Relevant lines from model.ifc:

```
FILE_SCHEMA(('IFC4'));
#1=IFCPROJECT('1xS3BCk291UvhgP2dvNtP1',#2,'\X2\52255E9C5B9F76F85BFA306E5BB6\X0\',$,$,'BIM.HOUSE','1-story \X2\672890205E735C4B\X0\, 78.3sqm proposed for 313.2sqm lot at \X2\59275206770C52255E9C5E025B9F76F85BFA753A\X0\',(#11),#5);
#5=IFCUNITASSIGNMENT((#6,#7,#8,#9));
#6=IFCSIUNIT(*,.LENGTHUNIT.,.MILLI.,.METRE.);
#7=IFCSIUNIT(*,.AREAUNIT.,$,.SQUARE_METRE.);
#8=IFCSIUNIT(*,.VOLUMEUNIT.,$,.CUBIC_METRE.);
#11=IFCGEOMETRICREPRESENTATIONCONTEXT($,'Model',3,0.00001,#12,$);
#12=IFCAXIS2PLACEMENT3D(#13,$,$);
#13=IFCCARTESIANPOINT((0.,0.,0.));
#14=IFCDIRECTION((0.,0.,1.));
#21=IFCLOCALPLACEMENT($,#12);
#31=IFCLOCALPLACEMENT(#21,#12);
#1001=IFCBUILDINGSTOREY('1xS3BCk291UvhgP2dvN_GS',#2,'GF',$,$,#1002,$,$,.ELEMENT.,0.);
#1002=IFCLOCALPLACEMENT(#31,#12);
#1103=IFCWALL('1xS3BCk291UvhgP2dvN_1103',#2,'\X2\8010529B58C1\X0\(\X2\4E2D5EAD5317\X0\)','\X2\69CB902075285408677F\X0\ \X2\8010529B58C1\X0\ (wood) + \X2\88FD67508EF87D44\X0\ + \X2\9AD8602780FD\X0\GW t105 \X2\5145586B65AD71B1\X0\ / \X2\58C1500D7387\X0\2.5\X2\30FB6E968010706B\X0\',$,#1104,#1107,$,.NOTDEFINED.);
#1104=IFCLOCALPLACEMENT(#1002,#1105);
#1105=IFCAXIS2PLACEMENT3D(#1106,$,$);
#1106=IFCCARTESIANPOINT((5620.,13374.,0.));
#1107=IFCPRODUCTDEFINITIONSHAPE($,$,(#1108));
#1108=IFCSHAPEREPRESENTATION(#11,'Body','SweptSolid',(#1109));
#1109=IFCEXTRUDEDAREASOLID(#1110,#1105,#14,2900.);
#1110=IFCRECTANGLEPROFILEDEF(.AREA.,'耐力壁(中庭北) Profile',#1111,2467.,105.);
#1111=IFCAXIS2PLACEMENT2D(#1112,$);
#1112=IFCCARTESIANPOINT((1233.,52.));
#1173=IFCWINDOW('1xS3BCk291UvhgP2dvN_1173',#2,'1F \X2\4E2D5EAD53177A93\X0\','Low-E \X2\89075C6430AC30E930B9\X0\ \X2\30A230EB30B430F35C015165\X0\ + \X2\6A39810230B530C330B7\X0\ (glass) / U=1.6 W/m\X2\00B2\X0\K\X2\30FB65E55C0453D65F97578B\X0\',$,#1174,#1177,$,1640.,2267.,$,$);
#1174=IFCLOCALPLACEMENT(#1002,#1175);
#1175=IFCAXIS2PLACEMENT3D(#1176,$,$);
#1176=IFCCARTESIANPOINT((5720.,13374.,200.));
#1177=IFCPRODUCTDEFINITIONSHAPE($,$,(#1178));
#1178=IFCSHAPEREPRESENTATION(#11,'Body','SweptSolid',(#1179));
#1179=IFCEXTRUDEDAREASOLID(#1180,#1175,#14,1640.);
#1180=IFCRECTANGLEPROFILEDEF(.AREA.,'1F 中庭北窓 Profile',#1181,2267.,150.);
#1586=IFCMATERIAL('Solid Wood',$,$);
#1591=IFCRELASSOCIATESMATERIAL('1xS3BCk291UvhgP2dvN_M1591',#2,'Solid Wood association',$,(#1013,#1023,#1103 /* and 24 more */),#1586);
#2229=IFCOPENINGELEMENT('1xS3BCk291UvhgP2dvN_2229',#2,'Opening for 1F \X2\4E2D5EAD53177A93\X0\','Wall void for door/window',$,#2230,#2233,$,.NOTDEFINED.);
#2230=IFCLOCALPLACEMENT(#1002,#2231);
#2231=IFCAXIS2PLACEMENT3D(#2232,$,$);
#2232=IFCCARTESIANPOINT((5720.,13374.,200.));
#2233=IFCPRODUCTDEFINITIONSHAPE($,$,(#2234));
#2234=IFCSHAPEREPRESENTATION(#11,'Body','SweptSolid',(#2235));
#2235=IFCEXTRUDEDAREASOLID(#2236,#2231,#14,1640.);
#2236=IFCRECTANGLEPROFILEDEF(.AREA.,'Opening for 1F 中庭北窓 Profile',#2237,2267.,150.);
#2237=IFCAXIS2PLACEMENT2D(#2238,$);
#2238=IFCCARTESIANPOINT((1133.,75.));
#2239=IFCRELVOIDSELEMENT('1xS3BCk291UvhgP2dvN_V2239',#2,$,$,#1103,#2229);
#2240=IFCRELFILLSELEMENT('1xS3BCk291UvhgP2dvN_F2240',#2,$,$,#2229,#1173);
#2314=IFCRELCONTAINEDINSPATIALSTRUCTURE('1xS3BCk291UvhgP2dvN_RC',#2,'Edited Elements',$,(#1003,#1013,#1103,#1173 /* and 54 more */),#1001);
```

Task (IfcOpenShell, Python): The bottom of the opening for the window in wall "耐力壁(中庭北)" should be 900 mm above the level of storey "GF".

```python
import numpy as np
import ifcopenshell
import ifcopenshell.api.geometry
import ifcopenshell.geom
import ifcopenshell.util.element
import ifcopenshell.util.placement
import ifcopenshell.util.shape
import ifcopenshell.util.unit

model = ifcopenshell.open("model.ifc")
unit_scale = ifcopenshell.util.unit.calculate_unit_scale(model)

window = model.by_id(1173)
opening = window.FillsVoids[0].RelatingOpeningElement
storey = ifcopenshell.util.element.get_container(window, ifc_class="IfcBuildingStorey")
level = ifcopenshell.util.placement.get_local_placement(storey.ObjectPlacement)[2, 3]

# The opening's origin need not be at the sill, so measure its lowest point.
shape = ifcopenshell.geom.create_shape(ifcopenshell.geom.settings(), opening)
bottom = ifcopenshell.util.shape.get_shape_bottom_elevation(shape, shape.geometry) / unit_scale
dz = level + 0.9 / unit_scale - bottom

shift = np.array([0.0, 0.0, dz])
# The window is not placed relative to its opening, so move both.
for product in (opening, window):
    matrix = ifcopenshell.util.placement.get_local_placement(product.ObjectPlacement)
    matrix[:3, 3] += shift
    ifcopenshell.api.geometry.edit_object_placement(model, product=product, matrix=matrix, is_si=False)

print(f"moved by {dz * unit_scale:+.3f} m")

model.write("model_updated.ifc")
```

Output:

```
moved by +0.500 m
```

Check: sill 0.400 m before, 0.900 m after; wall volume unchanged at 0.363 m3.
